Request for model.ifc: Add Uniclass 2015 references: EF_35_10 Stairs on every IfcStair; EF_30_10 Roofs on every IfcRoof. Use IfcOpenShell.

First a look at what the model holds.

```python
import ifcopenshell

model = ifcopenshell.open("model.ifc")
print(model.schema)
print("classifications:", [c.Name for c in model.by_type("IfcClassification")])
for ifc_class in ("IfcDoor", "IfcRoof", "IfcStair", "IfcWall", "IfcWindow"):
    print(ifc_class, len(model.by_type(ifc_class)))
```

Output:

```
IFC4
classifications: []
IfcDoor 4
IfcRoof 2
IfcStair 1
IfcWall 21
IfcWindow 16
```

```python
import ifcopenshell
import ifcopenshell.api.classification

model = ifcopenshell.open("model.ifc")

system = ifcopenshell.api.classification.add_classification(model, classification="Uniclass 2015")

codes = {
    "IfcStair": ("EF_35_10", "Stairs"),
    "IfcRoof": ("EF_30_10", "Roofs"),
}
for ifc_class, (code, name) in codes.items():
    products = model.by_type(ifc_class)
    ifcopenshell.api.classification.add_reference(
        model, products=products, classification=system, identification=code, name=name
    )
    print(code, len(products))

model.write("model_v2.ifc")
```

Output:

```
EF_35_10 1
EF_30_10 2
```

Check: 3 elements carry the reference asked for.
